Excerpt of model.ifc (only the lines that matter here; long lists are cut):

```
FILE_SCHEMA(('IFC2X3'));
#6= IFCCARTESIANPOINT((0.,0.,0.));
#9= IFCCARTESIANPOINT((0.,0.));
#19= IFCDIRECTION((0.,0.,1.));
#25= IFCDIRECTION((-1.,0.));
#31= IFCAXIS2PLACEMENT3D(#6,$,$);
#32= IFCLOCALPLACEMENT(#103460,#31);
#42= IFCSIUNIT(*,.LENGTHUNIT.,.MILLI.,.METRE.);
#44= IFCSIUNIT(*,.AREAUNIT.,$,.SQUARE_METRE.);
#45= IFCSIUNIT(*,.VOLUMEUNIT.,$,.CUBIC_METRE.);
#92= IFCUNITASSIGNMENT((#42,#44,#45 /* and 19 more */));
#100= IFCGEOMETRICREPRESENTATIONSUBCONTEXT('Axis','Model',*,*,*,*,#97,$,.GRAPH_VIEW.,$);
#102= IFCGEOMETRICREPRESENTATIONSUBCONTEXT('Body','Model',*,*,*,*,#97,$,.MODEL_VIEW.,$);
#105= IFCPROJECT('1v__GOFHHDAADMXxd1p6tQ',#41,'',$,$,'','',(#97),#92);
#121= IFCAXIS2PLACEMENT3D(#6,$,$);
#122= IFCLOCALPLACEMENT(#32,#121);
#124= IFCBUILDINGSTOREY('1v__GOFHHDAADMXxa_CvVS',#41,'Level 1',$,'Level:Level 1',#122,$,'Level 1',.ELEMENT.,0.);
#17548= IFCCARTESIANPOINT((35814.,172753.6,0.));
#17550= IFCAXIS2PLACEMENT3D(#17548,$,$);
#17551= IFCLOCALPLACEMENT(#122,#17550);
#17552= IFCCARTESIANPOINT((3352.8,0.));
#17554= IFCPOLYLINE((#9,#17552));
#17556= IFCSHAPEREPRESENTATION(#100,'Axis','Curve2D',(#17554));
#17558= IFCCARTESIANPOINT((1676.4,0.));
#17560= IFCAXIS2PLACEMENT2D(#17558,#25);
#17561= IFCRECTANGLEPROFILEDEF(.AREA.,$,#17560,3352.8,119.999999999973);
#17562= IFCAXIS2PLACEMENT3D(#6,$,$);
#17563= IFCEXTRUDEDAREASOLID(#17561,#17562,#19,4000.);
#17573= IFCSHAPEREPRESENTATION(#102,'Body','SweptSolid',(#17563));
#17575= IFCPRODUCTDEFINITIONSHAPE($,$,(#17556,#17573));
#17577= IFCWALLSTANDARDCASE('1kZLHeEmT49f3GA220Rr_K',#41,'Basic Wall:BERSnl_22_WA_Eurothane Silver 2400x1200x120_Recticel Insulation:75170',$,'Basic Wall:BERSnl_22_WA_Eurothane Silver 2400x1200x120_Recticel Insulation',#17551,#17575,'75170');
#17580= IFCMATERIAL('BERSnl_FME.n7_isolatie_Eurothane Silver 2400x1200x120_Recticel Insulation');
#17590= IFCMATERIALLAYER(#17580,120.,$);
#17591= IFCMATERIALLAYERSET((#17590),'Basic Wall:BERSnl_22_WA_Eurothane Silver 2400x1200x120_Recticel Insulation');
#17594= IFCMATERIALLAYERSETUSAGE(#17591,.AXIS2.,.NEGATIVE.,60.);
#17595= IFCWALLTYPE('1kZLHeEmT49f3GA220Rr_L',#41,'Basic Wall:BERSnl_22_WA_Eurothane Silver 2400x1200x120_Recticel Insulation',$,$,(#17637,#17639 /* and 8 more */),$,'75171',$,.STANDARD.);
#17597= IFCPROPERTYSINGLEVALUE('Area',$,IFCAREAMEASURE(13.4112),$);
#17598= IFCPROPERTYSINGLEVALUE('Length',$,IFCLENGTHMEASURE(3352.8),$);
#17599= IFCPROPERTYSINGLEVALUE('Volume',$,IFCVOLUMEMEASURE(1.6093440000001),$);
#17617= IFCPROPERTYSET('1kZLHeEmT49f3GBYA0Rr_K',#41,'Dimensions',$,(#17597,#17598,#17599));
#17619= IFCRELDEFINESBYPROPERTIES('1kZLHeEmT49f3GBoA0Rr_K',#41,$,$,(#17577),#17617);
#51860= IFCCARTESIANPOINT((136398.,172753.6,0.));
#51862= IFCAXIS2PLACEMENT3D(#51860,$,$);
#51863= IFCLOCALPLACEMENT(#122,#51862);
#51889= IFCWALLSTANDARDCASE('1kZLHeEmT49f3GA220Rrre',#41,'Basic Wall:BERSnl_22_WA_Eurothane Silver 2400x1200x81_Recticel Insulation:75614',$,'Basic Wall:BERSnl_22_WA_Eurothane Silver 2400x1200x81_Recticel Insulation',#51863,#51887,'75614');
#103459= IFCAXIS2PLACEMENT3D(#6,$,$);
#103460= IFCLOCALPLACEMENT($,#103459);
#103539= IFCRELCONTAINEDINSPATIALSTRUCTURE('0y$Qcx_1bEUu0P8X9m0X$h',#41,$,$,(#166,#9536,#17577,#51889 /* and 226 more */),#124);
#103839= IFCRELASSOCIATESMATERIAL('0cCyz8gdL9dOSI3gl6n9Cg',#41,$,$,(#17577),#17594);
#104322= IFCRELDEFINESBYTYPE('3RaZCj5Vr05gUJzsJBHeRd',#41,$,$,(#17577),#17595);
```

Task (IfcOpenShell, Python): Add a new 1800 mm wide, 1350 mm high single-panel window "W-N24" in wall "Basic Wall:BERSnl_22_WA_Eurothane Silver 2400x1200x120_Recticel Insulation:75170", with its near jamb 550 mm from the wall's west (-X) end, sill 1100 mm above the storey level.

```python
import numpy as np
import ifcopenshell
import ifcopenshell.api.feature
import ifcopenshell.api.geometry
import ifcopenshell.api.pset
import ifcopenshell.api.root
import ifcopenshell.api.spatial
import ifcopenshell.api.type
import ifcopenshell.geom
import ifcopenshell.util.element
import ifcopenshell.util.placement
import ifcopenshell.util.representation
import ifcopenshell.util.shape
import ifcopenshell.util.unit

model = ifcopenshell.open("model.ifc")
unit_scale = ifcopenshell.util.unit.calculate_unit_scale(model)
area_scale = ifcopenshell.util.unit.calculate_unit_scale(model, "AREAUNIT")
volume_scale = ifcopenshell.util.unit.calculate_unit_scale(model, "VOLUMEUNIT")
settings = ifcopenshell.geom.settings()


def volume(element):
    """Net volume in cubic metres, openings subtracted."""
    shape = ifcopenshell.geom.create_shape(settings, element)
    return ifcopenshell.util.shape.get_volume(shape.geometry)


wall = model.by_id(17577)
storey = ifcopenshell.util.element.get_container(wall, ifc_class="IfcBuildingStorey")
context = ifcopenshell.util.representation.get_context(model, "Model", "Body", "MODEL_VIEW")
before = volume(wall)

width, height, from_end, sill = 1.8, 1.35, 0.55, 1.1  # metres

# The wall runs along its own X axis, and the end named is its -X end.
wall_shape = ifcopenshell.geom.create_shape(settings, wall)
x, y, z = ifcopenshell.util.shape.get_vertices(wall_shape.geometry).T
start = x.min() + from_end
face, thickness = float(y.min()), float(y.max() - y.min())
wall_matrix = ifcopenshell.util.placement.get_local_placement(wall.ObjectPlacement)
level = ifcopenshell.util.placement.get_local_placement(storey.ObjectPlacement)[2, 3]


def in_wall(x, y):
    """Placement at x, y metres in the wall's axes, at sill height."""
    matrix = wall_matrix.copy()
    matrix[:, 3] = wall_matrix @ np.array([x / unit_scale, y / unit_scale, 0.0, 1.0])
    matrix[2, 3] = level + sill / unit_scale
    return matrix


# Opening: a box that overshoots both wall faces by 50 mm.
opening = ifcopenshell.api.root.create_entity(model, ifc_class="IfcOpeningElement")
box = ifcopenshell.api.geometry.add_wall_representation(
    model, context=context, length=width, height=height, thickness=thickness + 0.1
)
ifcopenshell.api.geometry.assign_representation(model, product=opening, representation=box)
ifcopenshell.api.geometry.edit_object_placement(model, product=opening, matrix=in_wall(start, face - 0.05), is_si=False)
ifcopenshell.api.feature.add_feature(model, feature=opening, element=wall)

window = ifcopenshell.api.root.create_entity(model, ifc_class="IfcWindow", name="W-N24")
window.OverallWidth, window.OverallHeight = width / unit_scale, height / unit_scale
body = ifcopenshell.api.geometry.add_window_representation(
    model,
    context=context,
    overall_width=window.OverallWidth,
    overall_height=window.OverallHeight,
    partition_type="SINGLE_PANEL",
)
ifcopenshell.api.geometry.assign_representation(model, product=window, representation=body)
ifcopenshell.api.spatial.assign_container(model, products=[window], relating_structure=storey)
fills = ifcopenshell.api.feature.add_filling(model, opening=opening, element=window)
fills.OwnerHistory = window.OwnerHistory  # required in IFC2X3

# IFC2X3 keeps the operation on the window style.
style = ifcopenshell.api.root.create_entity(model, ifc_class="IfcWindowStyle", name="W-N24")
style.OperationType, style.ConstructionType = "SINGLE_PANEL", "NOTDEFINED"
style.ParameterTakesPrecedence = style.Sizeable = False
ifcopenshell.api.type.assign_type(model, related_objects=[window], relating_type=style)

# Centre the window in the wall's thickness.
ifcopenshell.api.geometry.edit_object_placement(model, product=window, matrix=in_wall(start, face), is_si=False)
window_shape = ifcopenshell.geom.create_shape(settings, window)
depth = ifcopenshell.util.shape.get_vertices(window_shape.geometry)[:, 1]
offset = face + thickness / 2 - (depth.min() + depth.max()) / 2
ifcopenshell.api.geometry.edit_object_placement(model, product=window, matrix=in_wall(start, offset), is_si=False)

after = volume(wall)

# Update the wall's stored quantities.
pset = model.by_id(ifcopenshell.util.element.get_pset(wall, "Dimensions", should_inherit=False)["id"])
ifcopenshell.api.pset.edit_pset(model, pset=pset, properties={
    "Area": model.create_entity("IfcAreaMeasure", after / thickness / area_scale),
    "Volume": model.create_entity("IfcVolumeMeasure", after / volume_scale),
})

print(f"wall volume {before:.3f} -> {after:.3f} m3")

model.write("model-out.ifc")
```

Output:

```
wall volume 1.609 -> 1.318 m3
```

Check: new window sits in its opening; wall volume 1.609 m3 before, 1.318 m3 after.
